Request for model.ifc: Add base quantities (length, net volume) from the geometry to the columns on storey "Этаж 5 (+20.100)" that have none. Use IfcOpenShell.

First a look at what the model holds.

```python
import ifcopenshell
import ifcopenshell.util.element
import ifcopenshell.util.unit

model = ifcopenshell.open("model.ifc")
print(model.schema)
for unit_type in ("LENGTHUNIT", "AREAUNIT", "VOLUMEUNIT"):
    print(unit_type, ifcopenshell.util.unit.calculate_unit_scale(model, unit_type))
storey = next(s for s in model.by_type("IfcBuildingStorey") if s.Name == "Этаж 5 (+20.100)")
columns = [e for e in ifcopenshell.util.element.get_decomposition(storey) if e.is_a("IfcColumn")]
for e in sorted(columns, key=lambda e: e.id()):
    print(e.id(), e.is_a(), e.Name, list(ifcopenshell.util.element.get_psets(e, qtos_only=True)), sep=" | ")
```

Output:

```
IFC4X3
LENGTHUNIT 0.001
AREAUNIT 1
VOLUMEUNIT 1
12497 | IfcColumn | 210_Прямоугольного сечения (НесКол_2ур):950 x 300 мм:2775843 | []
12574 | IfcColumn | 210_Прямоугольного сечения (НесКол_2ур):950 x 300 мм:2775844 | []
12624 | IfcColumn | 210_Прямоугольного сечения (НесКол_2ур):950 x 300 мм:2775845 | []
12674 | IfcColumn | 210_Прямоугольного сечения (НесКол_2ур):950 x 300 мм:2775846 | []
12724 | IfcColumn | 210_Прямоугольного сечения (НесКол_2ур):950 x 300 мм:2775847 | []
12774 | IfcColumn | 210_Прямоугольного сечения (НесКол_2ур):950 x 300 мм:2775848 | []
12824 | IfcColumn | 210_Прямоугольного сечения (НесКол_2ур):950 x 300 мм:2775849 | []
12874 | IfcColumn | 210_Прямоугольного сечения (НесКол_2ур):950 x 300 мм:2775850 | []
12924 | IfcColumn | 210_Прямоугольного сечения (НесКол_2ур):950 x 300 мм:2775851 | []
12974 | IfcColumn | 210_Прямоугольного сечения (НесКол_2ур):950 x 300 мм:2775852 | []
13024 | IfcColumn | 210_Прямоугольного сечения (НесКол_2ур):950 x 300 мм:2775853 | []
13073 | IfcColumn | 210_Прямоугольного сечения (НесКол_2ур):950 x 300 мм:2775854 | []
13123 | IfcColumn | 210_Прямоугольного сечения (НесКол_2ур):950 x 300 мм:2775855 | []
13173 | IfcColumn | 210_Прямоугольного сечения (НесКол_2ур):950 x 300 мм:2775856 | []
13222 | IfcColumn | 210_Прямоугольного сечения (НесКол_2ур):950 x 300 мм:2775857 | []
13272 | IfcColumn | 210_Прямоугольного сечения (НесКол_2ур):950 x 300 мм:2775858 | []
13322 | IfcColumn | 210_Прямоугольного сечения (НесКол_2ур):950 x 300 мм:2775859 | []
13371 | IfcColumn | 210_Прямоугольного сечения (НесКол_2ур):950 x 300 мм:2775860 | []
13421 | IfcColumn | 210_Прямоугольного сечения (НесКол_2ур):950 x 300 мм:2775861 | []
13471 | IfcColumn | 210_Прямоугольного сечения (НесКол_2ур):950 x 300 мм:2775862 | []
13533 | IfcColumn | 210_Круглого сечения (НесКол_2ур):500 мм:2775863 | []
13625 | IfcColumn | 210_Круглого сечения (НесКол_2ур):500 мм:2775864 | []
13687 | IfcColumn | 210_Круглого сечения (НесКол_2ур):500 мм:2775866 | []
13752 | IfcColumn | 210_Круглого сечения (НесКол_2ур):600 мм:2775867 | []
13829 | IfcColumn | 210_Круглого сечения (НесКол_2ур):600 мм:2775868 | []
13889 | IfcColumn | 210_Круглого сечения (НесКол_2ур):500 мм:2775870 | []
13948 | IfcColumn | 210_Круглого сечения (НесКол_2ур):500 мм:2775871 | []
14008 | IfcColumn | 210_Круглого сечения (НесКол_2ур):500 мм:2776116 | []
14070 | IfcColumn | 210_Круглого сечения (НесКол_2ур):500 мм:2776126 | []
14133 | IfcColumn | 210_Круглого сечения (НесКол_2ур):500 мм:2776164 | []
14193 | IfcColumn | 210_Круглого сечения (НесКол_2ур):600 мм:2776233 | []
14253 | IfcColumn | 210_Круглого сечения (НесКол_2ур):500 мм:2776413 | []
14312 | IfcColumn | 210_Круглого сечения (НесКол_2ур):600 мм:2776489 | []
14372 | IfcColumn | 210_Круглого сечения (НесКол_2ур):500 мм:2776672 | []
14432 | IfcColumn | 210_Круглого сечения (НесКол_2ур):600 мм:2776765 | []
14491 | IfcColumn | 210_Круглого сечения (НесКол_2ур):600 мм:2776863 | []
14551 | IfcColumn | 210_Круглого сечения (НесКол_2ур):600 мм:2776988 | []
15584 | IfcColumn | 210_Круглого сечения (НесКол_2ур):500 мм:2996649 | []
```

```python
import ifcopenshell
import ifcopenshell.api.pset
import ifcopenshell.geom
import ifcopenshell.util.element
import ifcopenshell.util.shape
import ifcopenshell.util.unit

model = ifcopenshell.open("model.ifc")
unit_scale = ifcopenshell.util.unit.calculate_unit_scale(model)
volume_scale = ifcopenshell.util.unit.calculate_unit_scale(model, "VOLUMEUNIT")
settings = ifcopenshell.geom.settings()

storey = next(s for s in model.by_type("IfcBuildingStorey") if s.Name == "Этаж 5 (+20.100)")
columns = [e for e in ifcopenshell.util.element.get_decomposition(storey) if e.is_a("IfcColumn")]

for e in sorted(columns, key=lambda e: e.id()):
    if ifcopenshell.util.element.get_psets(e, qtos_only=True, should_inherit=False):
        continue
    # Geometry comes back in metres, in the element's own axes.
    shape = ifcopenshell.geom.create_shape(settings, e)
    values = {
        "Length": ifcopenshell.util.shape.get_z(shape.geometry) / unit_scale,
        "NetVolume": ifcopenshell.util.shape.get_volume(shape.geometry) / volume_scale,
    }
    qto = ifcopenshell.api.pset.add_qto(model, product=e, name="Qto_ColumnBaseQuantities")
    ifcopenshell.api.pset.edit_qto(model, qto=qto, properties=values)
    print(e.id(), {k: round(v, 3) for k, v in values.items()})

model.write("model-out.ifc")
```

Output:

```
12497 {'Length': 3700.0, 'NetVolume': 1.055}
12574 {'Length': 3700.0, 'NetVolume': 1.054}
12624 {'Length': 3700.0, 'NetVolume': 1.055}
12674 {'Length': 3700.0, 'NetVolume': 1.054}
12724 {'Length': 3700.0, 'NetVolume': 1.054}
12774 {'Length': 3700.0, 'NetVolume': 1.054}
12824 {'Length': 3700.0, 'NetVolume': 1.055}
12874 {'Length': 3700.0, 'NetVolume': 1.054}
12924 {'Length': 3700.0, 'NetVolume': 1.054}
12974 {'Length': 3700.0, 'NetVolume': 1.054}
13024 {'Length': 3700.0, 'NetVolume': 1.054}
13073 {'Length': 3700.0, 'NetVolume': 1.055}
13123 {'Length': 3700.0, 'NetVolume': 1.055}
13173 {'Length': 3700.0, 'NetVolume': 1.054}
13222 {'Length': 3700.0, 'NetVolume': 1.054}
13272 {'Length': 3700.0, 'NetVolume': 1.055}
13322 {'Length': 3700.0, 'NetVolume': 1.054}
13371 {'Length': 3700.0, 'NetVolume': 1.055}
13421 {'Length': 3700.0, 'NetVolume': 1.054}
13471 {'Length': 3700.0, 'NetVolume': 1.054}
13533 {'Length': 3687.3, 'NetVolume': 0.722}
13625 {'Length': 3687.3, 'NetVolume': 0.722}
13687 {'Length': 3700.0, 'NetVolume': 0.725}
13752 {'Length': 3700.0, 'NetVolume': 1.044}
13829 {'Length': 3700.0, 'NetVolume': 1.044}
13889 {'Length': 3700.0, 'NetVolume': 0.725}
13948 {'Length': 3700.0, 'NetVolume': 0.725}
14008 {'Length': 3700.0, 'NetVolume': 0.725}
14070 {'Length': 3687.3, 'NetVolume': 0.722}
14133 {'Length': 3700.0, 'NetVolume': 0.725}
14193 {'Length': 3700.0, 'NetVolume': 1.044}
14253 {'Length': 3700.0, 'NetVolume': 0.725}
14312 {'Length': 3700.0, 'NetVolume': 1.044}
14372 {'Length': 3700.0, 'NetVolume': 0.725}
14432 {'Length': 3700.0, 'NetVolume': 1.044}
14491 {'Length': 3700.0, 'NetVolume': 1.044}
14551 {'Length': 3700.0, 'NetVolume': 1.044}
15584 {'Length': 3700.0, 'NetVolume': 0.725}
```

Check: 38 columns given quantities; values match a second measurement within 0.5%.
